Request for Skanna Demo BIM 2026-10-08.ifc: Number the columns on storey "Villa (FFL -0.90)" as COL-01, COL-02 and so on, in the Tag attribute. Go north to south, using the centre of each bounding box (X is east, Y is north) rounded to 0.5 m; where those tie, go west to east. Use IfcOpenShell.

First a look at what the model holds.

```python
import ifcopenshell
import ifcopenshell.util.element
import ifcopenshell.util.placement

model = ifcopenshell.open("Skanna Demo BIM 2026-10-08.ifc")
print(model.schema)
storey = next(s for s in model.by_type("IfcBuildingStorey") if s.Name == "Villa (FFL -0.90)")
columns = [e for e in ifcopenshell.util.element.get_decomposition(storey) if e.is_a("IfcColumn")]
for e in sorted(columns, key=lambda e: e.id()):
    origin = ifcopenshell.util.placement.get_local_placement(e.ObjectPlacement)[:3, 3]
    print(e.id(), e.Tag, e.Name, origin.round(2) + 0.0, sep=" | ")
```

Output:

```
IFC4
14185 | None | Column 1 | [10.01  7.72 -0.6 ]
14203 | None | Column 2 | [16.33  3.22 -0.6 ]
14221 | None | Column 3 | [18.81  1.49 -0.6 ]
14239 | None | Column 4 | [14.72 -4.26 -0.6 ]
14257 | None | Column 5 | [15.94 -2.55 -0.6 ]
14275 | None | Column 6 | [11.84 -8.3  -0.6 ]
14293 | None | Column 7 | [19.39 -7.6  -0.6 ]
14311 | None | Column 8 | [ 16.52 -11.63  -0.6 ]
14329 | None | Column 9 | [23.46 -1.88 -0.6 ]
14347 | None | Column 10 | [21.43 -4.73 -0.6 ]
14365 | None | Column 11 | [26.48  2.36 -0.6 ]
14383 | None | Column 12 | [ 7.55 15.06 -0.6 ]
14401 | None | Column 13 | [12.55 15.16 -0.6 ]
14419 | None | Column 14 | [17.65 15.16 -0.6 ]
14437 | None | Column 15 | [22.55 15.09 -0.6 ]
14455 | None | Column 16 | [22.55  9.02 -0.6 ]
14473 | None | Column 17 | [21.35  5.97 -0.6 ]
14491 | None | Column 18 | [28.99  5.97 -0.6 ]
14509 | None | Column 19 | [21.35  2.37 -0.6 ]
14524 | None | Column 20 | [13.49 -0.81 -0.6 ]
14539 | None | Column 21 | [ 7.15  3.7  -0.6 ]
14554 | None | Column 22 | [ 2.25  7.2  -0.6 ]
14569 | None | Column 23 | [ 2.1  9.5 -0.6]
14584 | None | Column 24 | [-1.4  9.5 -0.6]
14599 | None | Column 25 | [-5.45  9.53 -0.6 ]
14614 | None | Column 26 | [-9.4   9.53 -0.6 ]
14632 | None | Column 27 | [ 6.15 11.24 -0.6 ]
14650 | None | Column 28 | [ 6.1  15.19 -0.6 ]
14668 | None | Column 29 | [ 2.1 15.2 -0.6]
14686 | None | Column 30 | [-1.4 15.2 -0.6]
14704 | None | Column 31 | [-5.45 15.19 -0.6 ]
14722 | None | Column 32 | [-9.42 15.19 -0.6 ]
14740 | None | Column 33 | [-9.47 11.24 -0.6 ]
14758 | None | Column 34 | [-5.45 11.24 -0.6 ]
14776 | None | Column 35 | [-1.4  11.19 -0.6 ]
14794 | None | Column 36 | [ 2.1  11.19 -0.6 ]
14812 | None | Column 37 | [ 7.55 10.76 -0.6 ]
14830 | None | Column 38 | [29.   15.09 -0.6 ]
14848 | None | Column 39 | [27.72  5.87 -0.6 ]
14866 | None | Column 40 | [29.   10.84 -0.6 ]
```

```python
import ifcopenshell
import ifcopenshell.geom
import ifcopenshell.util.element
import ifcopenshell.util.shape

model = ifcopenshell.open("Skanna Demo BIM 2026-10-08.ifc")
settings = ifcopenshell.geom.settings()
settings.set("use-world-coords", True)


def centre(element):
    shape = ifcopenshell.geom.create_shape(settings, element)
    return ifcopenshell.util.shape.get_bbox_centroid(shape.geometry)


storey = next(s for s in model.by_type("IfcBuildingStorey") if s.Name == "Villa (FFL -0.90)")
columns = [e for e in ifcopenshell.util.element.get_decomposition(storey) if e.is_a("IfcColumn")]

# Insertion points can sit at a corner or the storey origin, so sort by the geometry (in metres).
centres = {e: centre(e) for e in columns}
columns.sort(key=lambda e: (-round(centres[e][1] / 0.5), centres[e][0]))

for i, e in enumerate(columns, start=1):
    number = f"COL-{i:02d}"
    e.Tag = number
    print(e.id(), number)

model.write("Skanna Demo BIM 2026-10-08-out.ifc")
```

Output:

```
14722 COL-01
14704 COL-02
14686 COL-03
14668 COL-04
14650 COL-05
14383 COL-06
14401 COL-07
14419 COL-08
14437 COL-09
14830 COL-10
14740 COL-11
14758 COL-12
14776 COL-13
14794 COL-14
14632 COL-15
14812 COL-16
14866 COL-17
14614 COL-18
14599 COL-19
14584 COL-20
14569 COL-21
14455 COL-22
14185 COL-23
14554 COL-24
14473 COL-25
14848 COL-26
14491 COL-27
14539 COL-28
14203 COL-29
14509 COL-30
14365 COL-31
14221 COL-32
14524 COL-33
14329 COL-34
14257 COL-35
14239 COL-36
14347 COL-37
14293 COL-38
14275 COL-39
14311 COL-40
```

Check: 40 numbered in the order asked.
